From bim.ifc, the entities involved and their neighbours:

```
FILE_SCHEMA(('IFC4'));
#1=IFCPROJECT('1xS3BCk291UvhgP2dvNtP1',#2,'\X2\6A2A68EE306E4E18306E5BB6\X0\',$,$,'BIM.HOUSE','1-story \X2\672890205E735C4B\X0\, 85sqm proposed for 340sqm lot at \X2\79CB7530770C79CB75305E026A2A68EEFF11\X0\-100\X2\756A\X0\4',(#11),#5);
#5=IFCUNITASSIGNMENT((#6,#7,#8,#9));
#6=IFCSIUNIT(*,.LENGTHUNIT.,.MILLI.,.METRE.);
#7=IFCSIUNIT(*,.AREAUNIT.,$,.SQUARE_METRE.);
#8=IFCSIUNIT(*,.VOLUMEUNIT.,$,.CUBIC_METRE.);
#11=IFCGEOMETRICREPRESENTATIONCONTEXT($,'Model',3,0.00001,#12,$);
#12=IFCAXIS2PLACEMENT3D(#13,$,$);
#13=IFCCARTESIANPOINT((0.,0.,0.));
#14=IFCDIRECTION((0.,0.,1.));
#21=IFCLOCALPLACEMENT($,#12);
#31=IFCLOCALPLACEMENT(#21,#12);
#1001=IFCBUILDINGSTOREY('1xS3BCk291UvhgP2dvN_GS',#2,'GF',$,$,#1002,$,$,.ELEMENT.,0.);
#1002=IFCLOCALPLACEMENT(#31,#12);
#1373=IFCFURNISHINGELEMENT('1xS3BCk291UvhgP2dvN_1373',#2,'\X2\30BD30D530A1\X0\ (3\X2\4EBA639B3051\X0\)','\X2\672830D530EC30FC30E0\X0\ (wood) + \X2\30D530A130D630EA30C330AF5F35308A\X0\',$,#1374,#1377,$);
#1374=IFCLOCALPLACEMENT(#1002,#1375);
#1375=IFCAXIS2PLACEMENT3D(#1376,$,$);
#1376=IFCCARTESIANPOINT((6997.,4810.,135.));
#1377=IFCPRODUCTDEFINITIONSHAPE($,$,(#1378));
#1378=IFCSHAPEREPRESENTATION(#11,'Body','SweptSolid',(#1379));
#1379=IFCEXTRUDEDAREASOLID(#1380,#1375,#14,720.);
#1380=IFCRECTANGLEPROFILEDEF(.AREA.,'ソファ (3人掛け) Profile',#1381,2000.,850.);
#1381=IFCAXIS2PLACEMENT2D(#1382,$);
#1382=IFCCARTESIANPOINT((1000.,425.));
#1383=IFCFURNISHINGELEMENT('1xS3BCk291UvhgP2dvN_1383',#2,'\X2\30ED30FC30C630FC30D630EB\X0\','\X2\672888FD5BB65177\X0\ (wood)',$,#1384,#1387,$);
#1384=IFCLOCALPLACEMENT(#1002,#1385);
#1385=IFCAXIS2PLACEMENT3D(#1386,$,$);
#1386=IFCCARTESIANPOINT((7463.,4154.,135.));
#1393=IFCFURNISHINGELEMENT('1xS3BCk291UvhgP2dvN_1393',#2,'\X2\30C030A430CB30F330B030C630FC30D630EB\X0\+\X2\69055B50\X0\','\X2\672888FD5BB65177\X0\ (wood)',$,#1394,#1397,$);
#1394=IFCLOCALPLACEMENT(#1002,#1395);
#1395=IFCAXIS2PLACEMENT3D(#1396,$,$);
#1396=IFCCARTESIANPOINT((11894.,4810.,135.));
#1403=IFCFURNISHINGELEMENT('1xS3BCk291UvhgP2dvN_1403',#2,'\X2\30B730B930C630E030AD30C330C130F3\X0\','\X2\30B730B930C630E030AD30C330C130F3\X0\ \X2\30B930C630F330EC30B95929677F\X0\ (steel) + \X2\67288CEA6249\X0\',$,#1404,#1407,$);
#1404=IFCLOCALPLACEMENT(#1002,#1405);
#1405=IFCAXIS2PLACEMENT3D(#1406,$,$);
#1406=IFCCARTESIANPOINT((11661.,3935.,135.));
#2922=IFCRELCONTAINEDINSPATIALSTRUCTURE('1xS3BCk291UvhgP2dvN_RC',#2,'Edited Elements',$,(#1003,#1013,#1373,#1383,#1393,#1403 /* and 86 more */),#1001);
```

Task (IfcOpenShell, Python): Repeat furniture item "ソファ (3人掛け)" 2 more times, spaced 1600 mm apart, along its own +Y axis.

```python
import ifcopenshell
import ifcopenshell.api.geometry
import ifcopenshell.api.root
import ifcopenshell.util.element
import ifcopenshell.util.placement
import ifcopenshell.util.unit

model = ifcopenshell.open("bim.ifc")
unit_scale = ifcopenshell.util.unit.calculate_unit_scale(model)


def reuse_history(source, copy):
    """copy_class also copies each property set's owner history, people and application; keep the originals."""
    for rel in copy.IsDefinedBy:
        if rel.is_a("IfcRelDefinesByProperties") and (history := rel.RelatingPropertyDefinition.OwnerHistory):
            rel.RelatingPropertyDefinition.OwnerHistory = source.OwnerHistory
            ifcopenshell.util.element.remove_deep2(model, history)


source = model.by_id(1373)
base = ifcopenshell.util.placement.get_local_placement(source.ObjectPlacement)
step = base[:3, 1] * 1.6 / unit_scale

for i in range(1, 3):
    copy = ifcopenshell.api.root.copy_class(model, product=source)
    copy.Representation = ifcopenshell.util.element.copy_deep(
        model, source.Representation, exclude=["IfcGeometricRepresentationContext", "IfcRepresentationMap"]
    )
    reuse_history(source, copy)
    matrix = base.copy()
    matrix[:3, 3] += i * step
    print("added at", matrix[:3, 3].round(3) + 0.0)
    ifcopenshell.api.geometry.edit_object_placement(model, product=copy, matrix=matrix, is_si=False)

model.write("bim_edited.ifc")
```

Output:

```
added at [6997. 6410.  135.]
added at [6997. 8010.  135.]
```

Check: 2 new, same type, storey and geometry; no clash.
